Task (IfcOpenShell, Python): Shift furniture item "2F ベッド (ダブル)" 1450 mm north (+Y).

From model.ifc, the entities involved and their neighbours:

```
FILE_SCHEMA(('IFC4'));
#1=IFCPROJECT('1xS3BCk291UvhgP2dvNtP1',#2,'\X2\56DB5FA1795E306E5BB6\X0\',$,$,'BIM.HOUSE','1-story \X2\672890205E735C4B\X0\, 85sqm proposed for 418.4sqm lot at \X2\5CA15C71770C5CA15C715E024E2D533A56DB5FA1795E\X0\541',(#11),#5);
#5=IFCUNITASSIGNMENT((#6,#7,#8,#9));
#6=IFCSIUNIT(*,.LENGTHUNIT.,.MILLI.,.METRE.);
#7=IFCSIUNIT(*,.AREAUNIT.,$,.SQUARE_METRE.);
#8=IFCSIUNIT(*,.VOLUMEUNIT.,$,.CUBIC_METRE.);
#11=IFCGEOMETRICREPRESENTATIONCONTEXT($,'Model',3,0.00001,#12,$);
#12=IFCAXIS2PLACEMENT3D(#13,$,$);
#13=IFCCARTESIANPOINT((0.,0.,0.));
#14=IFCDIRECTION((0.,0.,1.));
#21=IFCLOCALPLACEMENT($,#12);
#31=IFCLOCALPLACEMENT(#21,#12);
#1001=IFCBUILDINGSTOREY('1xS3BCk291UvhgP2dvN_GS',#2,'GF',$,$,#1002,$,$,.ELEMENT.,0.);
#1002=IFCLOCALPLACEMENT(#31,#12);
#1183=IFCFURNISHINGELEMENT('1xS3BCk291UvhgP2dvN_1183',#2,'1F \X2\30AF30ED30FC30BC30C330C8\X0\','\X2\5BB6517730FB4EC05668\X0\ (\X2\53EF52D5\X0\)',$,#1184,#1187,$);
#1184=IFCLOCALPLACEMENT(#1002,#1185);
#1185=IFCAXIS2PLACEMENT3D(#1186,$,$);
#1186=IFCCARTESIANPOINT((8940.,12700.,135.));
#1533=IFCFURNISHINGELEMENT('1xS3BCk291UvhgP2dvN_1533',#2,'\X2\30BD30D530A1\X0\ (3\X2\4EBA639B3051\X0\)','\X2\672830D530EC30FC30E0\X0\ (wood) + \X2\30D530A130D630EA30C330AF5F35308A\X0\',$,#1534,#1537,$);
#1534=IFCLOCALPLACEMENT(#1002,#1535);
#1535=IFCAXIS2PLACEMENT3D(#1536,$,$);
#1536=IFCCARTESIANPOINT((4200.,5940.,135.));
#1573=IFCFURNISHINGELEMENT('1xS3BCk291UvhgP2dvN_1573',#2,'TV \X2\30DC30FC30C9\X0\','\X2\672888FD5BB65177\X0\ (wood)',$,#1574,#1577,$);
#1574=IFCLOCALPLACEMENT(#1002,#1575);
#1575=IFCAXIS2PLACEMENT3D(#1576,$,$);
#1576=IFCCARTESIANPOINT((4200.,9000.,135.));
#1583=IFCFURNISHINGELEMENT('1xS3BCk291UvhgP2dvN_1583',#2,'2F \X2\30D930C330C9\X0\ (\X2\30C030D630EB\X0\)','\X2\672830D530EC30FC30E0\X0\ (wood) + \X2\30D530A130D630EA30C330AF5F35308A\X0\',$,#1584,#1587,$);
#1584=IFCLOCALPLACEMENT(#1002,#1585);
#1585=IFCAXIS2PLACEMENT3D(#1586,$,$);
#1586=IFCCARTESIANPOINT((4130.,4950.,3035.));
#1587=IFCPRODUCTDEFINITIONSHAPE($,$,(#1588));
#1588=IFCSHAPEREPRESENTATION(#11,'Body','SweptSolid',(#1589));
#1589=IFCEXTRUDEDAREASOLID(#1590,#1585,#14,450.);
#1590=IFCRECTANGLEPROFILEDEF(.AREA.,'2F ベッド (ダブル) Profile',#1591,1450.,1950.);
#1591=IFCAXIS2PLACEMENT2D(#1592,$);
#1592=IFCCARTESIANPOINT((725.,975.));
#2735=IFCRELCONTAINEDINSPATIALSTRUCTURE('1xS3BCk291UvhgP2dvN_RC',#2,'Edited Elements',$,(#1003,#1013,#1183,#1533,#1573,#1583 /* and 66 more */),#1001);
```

```python
import ifcopenshell
import ifcopenshell.api.geometry
import ifcopenshell.util.placement

model = ifcopenshell.open("model.ifc")

item = model.by_guid("1xS3BCk291UvhgP2dvN_1583")
matrix = ifcopenshell.util.placement.get_local_placement(item.ObjectPlacement)
matrix[1, 3] += 1450.0
ifcopenshell.api.geometry.edit_object_placement(model, product=item, matrix=matrix, is_si=False)

print(ifcopenshell.util.placement.get_local_placement(item.ObjectPlacement).round(3) + 0.0)

model.write("model_rev.ifc")
```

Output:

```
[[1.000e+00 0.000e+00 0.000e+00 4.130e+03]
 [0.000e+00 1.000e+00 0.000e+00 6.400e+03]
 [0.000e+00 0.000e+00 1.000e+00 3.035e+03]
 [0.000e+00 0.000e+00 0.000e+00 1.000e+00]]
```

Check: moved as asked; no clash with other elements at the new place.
